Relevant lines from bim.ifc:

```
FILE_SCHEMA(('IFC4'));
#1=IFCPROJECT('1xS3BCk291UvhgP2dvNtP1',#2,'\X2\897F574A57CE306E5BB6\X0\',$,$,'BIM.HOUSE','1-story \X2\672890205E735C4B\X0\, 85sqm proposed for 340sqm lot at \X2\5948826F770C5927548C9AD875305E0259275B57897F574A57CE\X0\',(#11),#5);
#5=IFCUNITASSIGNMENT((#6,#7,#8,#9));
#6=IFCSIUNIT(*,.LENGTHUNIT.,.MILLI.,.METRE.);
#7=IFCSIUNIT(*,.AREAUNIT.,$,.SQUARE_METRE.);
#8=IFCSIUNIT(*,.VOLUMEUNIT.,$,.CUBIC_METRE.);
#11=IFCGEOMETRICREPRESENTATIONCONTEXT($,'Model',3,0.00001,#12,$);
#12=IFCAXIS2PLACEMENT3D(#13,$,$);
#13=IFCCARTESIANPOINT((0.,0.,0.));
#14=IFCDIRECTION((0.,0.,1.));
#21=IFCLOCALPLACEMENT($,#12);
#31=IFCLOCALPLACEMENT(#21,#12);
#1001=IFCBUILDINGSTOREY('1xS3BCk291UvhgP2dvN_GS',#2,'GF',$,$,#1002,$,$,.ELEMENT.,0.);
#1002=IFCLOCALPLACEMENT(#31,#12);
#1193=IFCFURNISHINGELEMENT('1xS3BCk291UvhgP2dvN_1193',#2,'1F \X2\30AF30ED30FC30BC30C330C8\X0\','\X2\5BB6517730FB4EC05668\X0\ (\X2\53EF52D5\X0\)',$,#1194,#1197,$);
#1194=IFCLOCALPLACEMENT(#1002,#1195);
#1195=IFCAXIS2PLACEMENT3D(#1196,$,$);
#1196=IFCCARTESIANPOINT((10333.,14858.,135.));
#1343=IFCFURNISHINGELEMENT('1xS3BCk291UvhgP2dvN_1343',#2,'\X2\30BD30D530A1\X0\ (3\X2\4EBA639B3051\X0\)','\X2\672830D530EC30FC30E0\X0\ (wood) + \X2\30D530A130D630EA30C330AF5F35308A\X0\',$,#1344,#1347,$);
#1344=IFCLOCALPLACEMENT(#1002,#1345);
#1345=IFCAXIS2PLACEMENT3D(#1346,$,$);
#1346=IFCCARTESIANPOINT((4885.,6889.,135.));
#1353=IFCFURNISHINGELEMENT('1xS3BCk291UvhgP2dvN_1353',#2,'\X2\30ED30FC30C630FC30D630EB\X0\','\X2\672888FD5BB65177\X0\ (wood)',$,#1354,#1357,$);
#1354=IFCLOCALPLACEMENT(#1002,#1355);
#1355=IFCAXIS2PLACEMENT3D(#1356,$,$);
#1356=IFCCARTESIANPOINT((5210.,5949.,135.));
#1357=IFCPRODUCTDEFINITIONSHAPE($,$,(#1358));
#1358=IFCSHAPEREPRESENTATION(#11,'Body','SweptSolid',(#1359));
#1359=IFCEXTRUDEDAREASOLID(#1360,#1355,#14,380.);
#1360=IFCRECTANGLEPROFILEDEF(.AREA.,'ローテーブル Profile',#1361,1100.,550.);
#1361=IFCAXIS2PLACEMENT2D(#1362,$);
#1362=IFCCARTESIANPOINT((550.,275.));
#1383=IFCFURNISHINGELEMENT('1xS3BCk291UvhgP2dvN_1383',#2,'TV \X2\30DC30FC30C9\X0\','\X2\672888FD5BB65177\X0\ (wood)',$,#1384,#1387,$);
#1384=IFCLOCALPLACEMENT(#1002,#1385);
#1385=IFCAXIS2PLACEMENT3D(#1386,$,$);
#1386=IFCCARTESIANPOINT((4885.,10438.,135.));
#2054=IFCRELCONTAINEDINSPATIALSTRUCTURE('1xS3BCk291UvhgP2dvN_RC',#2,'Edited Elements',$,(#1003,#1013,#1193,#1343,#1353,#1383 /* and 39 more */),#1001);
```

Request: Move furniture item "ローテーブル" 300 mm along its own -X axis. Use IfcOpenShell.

```python
import ifcopenshell
import ifcopenshell.api.geometry
import ifcopenshell.util.placement
import ifcopenshell.util.unit

model = ifcopenshell.open("bim.ifc")
unit_scale = ifcopenshell.util.unit.calculate_unit_scale(model)

item = model.by_guid("1xS3BCk291UvhgP2dvN_1353")
matrix = ifcopenshell.util.placement.get_local_placement(item.ObjectPlacement)
matrix[:3, 3] -= matrix[:3, 0] * 0.3 / unit_scale
ifcopenshell.api.geometry.edit_object_placement(model, product=item, matrix=matrix, is_si=False)

print(ifcopenshell.util.placement.get_local_placement(item.ObjectPlacement).round(3) + 0.0)

model.write("bim_v2.ifc")
```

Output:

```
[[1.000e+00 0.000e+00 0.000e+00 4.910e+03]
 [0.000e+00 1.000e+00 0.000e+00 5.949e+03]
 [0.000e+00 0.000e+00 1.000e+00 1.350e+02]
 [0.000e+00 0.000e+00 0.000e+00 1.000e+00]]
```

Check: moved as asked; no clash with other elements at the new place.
